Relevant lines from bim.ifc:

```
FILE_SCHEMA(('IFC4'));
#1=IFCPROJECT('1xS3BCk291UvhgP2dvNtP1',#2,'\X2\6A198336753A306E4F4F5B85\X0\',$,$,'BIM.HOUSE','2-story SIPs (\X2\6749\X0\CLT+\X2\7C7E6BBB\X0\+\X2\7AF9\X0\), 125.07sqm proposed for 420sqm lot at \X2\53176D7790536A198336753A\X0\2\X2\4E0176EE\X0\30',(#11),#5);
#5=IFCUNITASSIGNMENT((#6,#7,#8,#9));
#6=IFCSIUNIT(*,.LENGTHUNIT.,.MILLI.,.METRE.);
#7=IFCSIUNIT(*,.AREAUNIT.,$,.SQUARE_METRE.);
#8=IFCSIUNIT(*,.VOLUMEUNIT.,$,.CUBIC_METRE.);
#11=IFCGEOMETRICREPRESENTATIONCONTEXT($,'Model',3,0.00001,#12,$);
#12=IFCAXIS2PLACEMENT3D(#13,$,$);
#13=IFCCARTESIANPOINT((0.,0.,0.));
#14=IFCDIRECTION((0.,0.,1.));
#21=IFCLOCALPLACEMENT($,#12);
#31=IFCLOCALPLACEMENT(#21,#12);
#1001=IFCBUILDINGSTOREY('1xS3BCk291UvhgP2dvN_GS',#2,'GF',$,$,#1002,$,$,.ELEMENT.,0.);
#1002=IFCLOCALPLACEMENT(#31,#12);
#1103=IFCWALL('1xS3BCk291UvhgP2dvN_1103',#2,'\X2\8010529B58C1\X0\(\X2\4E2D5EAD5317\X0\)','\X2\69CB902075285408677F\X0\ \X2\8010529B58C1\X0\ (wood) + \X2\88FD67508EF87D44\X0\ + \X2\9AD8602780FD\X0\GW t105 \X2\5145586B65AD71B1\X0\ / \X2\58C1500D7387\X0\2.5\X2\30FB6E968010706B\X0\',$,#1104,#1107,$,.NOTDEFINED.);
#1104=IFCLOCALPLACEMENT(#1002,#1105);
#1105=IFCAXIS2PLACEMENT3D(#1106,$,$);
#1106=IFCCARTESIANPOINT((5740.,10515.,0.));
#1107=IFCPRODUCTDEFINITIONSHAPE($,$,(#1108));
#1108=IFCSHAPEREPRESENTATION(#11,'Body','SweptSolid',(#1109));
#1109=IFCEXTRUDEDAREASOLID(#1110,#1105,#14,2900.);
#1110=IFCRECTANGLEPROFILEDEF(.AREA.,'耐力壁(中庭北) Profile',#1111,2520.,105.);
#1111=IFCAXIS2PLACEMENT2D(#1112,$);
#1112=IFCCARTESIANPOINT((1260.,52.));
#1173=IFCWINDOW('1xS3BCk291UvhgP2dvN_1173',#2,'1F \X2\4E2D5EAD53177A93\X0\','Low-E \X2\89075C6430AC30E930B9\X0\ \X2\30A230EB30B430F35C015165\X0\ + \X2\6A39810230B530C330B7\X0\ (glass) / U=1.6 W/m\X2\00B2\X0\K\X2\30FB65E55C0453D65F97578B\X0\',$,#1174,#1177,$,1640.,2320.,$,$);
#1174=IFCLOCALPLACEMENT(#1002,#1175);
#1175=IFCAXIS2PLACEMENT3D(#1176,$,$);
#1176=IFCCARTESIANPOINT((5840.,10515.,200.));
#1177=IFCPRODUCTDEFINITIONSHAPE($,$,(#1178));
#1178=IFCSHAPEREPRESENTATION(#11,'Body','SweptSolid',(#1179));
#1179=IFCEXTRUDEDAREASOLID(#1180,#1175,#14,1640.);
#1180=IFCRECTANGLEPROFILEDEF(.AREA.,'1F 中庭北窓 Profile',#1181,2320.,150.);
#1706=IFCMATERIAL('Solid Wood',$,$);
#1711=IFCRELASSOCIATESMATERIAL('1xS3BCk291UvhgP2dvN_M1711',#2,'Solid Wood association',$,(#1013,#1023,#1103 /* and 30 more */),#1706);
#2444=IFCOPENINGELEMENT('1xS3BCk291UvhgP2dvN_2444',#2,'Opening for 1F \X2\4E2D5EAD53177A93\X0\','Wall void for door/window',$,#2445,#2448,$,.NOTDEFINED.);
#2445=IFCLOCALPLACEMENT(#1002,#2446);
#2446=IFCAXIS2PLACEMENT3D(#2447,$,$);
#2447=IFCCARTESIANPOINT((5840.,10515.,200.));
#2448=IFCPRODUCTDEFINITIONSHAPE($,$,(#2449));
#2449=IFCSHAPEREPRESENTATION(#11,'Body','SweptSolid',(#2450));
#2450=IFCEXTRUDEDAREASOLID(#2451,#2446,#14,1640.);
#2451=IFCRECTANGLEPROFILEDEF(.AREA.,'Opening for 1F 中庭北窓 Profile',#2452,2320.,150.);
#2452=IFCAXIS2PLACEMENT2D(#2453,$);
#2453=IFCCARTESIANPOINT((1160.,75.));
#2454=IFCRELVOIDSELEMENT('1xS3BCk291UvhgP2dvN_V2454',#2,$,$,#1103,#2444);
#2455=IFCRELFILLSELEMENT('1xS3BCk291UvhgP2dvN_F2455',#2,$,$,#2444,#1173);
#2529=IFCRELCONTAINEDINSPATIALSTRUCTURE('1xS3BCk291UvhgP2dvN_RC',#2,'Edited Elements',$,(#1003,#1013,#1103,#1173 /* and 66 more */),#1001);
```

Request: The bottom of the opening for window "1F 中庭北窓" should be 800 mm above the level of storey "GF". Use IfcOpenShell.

```python
import numpy as np
import ifcopenshell
import ifcopenshell.api.geometry
import ifcopenshell.geom
import ifcopenshell.util.element
import ifcopenshell.util.placement
import ifcopenshell.util.shape
import ifcopenshell.util.unit

model = ifcopenshell.open("bim.ifc")
unit_scale = ifcopenshell.util.unit.calculate_unit_scale(model)

window = model.by_guid("1xS3BCk291UvhgP2dvN_1173")
opening = window.FillsVoids[0].RelatingOpeningElement
storey = ifcopenshell.util.element.get_container(window, ifc_class="IfcBuildingStorey")
level = ifcopenshell.util.placement.get_local_placement(storey.ObjectPlacement)[2, 3]

# The opening's origin need not be at the sill, so measure its lowest point.
shape = ifcopenshell.geom.create_shape(ifcopenshell.geom.settings(), opening)
bottom = ifcopenshell.util.shape.get_shape_bottom_elevation(shape, shape.geometry) / unit_scale
dz = level + 800.0 - bottom

shift = np.array([0.0, 0.0, dz])
# The window is not placed relative to its opening, so move both.
for product in (opening, window):
    matrix = ifcopenshell.util.placement.get_local_placement(product.ObjectPlacement)
    matrix[:3, 3] += shift
    ifcopenshell.api.geometry.edit_object_placement(model, product=product, matrix=matrix, is_si=False)

print(f"moved by {dz * unit_scale:+.3f} m")

model.write("bim-out.ifc")
```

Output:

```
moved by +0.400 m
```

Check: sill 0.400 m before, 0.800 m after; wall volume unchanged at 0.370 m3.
